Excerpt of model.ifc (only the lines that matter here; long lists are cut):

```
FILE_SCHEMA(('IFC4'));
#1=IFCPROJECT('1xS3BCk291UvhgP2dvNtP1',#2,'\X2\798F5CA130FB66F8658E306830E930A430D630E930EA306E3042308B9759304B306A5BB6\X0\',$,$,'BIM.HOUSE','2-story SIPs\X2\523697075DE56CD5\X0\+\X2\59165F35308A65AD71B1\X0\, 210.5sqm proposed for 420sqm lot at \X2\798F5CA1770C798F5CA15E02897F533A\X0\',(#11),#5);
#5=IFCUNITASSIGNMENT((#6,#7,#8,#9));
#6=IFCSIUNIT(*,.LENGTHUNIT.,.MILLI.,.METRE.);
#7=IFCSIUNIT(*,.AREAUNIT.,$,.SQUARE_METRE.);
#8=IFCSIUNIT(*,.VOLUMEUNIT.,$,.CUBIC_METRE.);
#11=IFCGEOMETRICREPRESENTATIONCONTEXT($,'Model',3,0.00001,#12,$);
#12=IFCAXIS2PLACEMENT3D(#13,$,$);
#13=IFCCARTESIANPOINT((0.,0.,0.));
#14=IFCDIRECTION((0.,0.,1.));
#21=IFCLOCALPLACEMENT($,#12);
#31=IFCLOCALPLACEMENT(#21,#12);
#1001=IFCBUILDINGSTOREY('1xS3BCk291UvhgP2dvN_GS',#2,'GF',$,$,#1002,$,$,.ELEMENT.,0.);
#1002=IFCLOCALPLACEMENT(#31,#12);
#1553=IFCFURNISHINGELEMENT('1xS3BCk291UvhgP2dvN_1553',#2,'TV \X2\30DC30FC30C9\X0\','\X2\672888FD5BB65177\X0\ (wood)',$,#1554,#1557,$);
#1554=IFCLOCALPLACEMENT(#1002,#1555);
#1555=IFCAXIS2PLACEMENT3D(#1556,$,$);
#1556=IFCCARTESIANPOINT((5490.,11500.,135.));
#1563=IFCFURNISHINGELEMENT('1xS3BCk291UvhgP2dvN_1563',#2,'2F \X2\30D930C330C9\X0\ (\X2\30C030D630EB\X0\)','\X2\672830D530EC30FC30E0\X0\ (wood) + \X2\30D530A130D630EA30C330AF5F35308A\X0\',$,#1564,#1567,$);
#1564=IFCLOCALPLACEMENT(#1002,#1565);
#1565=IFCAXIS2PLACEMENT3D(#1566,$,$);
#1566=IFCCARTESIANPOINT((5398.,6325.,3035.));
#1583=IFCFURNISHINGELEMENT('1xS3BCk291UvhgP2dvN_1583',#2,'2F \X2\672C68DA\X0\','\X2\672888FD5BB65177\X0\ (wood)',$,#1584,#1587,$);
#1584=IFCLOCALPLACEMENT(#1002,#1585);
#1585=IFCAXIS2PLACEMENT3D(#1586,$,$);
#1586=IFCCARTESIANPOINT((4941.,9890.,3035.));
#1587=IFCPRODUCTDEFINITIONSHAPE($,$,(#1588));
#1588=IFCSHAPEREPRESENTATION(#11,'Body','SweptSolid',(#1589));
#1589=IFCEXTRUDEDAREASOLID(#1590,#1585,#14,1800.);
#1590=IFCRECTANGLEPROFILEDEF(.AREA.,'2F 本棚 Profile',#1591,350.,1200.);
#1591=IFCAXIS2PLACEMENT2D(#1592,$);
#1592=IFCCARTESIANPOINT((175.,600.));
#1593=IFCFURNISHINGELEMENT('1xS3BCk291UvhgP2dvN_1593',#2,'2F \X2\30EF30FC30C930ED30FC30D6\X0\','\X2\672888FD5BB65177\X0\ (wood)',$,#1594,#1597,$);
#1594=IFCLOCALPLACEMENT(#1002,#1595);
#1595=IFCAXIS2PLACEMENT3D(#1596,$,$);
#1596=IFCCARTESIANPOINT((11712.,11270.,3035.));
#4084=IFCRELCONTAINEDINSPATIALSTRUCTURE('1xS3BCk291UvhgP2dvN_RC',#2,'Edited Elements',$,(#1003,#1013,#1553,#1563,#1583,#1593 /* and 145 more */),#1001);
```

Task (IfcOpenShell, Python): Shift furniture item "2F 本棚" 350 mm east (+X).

```python
import ifcopenshell
import ifcopenshell.api.geometry
import ifcopenshell.util.placement

model = ifcopenshell.open("model.ifc")

item = model.by_id(1583)
matrix = ifcopenshell.util.placement.get_local_placement(item.ObjectPlacement)
matrix[0, 3] += 350.0
ifcopenshell.api.geometry.edit_object_placement(model, product=item, matrix=matrix, is_si=False)

print(ifcopenshell.util.placement.get_local_placement(item.ObjectPlacement).round(3) + 0.0)

model.write("model_updated.ifc")
```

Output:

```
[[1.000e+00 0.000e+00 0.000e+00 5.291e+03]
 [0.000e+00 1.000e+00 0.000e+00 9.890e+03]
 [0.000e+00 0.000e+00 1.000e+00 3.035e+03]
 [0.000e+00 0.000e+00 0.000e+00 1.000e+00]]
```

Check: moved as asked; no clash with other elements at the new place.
